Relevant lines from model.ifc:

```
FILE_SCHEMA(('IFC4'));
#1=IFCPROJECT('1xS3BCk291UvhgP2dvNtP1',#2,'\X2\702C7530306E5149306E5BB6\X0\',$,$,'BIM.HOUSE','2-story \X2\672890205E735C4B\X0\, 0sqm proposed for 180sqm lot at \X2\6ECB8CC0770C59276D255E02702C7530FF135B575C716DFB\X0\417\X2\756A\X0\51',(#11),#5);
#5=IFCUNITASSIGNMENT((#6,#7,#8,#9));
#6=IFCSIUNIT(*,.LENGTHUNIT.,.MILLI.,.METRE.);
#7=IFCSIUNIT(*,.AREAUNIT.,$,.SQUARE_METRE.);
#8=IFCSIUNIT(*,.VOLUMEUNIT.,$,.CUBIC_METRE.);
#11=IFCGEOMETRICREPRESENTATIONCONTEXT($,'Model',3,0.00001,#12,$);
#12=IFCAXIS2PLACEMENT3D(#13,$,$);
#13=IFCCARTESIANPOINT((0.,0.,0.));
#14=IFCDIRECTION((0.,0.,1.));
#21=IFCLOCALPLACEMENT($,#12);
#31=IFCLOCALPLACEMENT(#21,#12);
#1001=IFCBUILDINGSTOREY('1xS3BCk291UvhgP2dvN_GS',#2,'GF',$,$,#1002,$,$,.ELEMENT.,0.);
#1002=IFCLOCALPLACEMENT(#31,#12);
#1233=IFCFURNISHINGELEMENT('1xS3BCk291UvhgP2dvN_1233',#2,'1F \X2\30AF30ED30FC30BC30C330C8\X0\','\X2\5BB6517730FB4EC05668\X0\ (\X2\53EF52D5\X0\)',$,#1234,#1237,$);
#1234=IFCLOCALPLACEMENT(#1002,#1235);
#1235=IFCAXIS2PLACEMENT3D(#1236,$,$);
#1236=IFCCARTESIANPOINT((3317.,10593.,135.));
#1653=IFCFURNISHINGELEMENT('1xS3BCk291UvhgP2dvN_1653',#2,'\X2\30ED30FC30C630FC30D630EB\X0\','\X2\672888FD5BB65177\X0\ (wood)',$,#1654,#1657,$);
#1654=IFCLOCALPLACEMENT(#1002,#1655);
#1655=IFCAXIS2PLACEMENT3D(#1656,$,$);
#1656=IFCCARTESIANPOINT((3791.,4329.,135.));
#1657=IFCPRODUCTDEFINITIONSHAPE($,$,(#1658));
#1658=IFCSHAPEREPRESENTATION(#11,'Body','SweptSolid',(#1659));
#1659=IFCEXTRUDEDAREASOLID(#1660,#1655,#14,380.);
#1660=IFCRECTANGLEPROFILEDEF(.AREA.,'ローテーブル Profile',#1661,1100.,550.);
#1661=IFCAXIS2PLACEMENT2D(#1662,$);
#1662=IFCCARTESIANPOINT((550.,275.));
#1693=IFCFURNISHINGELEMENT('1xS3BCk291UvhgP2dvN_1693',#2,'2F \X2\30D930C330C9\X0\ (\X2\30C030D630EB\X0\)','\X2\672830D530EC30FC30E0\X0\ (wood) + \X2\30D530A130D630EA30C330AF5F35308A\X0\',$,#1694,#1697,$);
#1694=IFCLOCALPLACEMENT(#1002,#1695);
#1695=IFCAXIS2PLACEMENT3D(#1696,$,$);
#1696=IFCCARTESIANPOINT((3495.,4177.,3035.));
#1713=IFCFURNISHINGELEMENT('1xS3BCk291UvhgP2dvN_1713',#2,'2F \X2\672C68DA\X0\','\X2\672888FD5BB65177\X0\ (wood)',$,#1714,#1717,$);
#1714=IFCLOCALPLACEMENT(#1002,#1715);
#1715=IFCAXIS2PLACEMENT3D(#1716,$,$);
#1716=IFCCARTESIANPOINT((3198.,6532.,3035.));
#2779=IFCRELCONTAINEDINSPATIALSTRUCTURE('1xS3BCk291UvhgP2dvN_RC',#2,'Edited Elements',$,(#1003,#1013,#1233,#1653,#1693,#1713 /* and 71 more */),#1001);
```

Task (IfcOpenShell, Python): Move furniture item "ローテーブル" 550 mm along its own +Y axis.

```python
import ifcopenshell
import ifcopenshell.api.geometry
import ifcopenshell.util.placement
import ifcopenshell.util.unit

model = ifcopenshell.open("model.ifc")
unit_scale = ifcopenshell.util.unit.calculate_unit_scale(model)

item = model.by_guid("1xS3BCk291UvhgP2dvN_1653")
matrix = ifcopenshell.util.placement.get_local_placement(item.ObjectPlacement)
matrix[:3, 3] += matrix[:3, 1] * 0.55 / unit_scale
ifcopenshell.api.geometry.edit_object_placement(model, product=item, matrix=matrix, is_si=False)

print(ifcopenshell.util.placement.get_local_placement(item.ObjectPlacement).round(3) + 0.0)

model.write("model_rev.ifc")
```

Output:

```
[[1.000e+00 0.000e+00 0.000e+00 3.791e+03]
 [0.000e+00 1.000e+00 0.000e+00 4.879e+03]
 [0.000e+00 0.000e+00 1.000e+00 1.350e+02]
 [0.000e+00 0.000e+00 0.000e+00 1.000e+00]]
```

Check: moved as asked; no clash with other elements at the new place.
